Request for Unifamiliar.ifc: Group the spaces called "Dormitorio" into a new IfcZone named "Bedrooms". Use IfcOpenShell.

First a look at what the model holds.

```python
import ifcopenshell

model = ifcopenshell.open("Unifamiliar.ifc")
print(model.schema)
seen = {}
for space in model.by_type("IfcSpace"):
    seen[space.LongName] = seen.get(space.LongName, 0) + 1
for name, count in sorted(seen.items(), key=str):
    print(count, "x", name)
print("zones:", [z.Name for z in model.by_type("IfcZone")][:20])
```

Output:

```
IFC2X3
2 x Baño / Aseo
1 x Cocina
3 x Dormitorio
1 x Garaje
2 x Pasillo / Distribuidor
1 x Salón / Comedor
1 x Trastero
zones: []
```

```python
import ifcopenshell
import ifcopenshell.api.group
import ifcopenshell.api.root

model = ifcopenshell.open("Unifamiliar.ifc")

names = {"Dormitorio"}
spaces = [s for s in model.by_type("IfcSpace") if s.LongName in names]

zone = ifcopenshell.api.root.create_entity(model, ifc_class="IfcZone", name="Bedrooms")
ifcopenshell.api.group.assign_group(model, products=spaces, group=zone)
print(len(spaces), "spaces in", zone.Name)

model.write("Unifamiliar_updated.ifc")
```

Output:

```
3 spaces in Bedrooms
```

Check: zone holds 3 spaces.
